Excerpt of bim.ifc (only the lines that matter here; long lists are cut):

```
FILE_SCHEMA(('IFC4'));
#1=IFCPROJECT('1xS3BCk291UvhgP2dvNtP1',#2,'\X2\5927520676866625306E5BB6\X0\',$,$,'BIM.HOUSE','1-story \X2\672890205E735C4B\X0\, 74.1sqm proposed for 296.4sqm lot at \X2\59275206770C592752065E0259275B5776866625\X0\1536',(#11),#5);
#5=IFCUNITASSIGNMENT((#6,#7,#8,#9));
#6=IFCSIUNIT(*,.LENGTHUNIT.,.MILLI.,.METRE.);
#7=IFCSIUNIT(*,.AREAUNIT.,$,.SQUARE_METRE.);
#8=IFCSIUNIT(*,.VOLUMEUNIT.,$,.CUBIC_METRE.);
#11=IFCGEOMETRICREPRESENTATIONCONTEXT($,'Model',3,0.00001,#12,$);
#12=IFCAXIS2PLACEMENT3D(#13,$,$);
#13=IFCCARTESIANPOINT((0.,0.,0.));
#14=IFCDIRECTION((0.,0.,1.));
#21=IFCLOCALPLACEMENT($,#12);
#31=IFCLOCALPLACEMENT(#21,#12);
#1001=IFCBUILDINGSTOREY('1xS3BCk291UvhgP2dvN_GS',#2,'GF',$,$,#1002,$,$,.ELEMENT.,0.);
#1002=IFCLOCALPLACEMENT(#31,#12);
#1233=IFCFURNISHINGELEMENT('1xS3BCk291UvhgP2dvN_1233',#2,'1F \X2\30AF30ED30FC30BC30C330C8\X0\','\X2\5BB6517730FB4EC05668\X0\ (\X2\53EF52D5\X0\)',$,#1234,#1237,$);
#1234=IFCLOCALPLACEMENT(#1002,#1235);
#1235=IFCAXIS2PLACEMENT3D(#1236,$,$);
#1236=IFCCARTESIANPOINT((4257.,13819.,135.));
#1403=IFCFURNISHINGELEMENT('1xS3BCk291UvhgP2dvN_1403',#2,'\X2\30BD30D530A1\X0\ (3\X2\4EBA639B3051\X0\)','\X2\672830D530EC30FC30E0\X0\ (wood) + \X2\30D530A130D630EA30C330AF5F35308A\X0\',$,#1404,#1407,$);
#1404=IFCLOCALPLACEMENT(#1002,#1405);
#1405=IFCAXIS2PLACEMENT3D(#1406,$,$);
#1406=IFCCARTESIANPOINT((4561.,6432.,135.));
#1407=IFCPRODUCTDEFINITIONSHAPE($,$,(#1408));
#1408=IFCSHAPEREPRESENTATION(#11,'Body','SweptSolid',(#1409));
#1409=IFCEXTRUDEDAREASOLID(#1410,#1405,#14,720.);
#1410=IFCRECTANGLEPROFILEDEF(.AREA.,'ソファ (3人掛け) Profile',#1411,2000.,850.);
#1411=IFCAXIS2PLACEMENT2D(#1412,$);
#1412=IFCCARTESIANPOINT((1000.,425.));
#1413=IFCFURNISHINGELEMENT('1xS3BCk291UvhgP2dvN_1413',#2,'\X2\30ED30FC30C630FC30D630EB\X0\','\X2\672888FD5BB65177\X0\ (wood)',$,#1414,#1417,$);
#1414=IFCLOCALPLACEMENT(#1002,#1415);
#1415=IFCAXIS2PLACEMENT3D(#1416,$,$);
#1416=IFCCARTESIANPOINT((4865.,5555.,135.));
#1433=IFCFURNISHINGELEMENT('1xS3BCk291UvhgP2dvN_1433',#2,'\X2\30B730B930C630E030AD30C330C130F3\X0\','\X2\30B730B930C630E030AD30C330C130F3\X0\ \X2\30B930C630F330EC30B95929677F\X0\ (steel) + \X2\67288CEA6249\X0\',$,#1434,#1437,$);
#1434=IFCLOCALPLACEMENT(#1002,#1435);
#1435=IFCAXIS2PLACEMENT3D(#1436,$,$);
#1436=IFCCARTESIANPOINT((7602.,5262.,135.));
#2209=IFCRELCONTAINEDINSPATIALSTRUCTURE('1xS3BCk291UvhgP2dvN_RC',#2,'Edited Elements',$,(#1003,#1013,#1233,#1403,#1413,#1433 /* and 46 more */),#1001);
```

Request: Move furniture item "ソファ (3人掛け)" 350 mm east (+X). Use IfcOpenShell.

```python
import ifcopenshell
import ifcopenshell.api.geometry
import ifcopenshell.util.placement
import ifcopenshell.util.unit

model = ifcopenshell.open("bim.ifc")
unit_scale = ifcopenshell.util.unit.calculate_unit_scale(model)

item = model.by_guid("1xS3BCk291UvhgP2dvN_1403")
matrix = ifcopenshell.util.placement.get_local_placement(item.ObjectPlacement)
matrix[0, 3] += 0.35 / unit_scale
ifcopenshell.api.geometry.edit_object_placement(model, product=item, matrix=matrix, is_si=False)

print(ifcopenshell.util.placement.get_local_placement(item.ObjectPlacement).round(3) + 0.0)

model.write("bim-out.ifc")
```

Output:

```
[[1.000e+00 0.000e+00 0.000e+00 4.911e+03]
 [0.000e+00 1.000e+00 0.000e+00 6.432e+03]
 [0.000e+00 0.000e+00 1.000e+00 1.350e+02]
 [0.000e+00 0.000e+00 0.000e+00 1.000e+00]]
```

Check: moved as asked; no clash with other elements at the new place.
